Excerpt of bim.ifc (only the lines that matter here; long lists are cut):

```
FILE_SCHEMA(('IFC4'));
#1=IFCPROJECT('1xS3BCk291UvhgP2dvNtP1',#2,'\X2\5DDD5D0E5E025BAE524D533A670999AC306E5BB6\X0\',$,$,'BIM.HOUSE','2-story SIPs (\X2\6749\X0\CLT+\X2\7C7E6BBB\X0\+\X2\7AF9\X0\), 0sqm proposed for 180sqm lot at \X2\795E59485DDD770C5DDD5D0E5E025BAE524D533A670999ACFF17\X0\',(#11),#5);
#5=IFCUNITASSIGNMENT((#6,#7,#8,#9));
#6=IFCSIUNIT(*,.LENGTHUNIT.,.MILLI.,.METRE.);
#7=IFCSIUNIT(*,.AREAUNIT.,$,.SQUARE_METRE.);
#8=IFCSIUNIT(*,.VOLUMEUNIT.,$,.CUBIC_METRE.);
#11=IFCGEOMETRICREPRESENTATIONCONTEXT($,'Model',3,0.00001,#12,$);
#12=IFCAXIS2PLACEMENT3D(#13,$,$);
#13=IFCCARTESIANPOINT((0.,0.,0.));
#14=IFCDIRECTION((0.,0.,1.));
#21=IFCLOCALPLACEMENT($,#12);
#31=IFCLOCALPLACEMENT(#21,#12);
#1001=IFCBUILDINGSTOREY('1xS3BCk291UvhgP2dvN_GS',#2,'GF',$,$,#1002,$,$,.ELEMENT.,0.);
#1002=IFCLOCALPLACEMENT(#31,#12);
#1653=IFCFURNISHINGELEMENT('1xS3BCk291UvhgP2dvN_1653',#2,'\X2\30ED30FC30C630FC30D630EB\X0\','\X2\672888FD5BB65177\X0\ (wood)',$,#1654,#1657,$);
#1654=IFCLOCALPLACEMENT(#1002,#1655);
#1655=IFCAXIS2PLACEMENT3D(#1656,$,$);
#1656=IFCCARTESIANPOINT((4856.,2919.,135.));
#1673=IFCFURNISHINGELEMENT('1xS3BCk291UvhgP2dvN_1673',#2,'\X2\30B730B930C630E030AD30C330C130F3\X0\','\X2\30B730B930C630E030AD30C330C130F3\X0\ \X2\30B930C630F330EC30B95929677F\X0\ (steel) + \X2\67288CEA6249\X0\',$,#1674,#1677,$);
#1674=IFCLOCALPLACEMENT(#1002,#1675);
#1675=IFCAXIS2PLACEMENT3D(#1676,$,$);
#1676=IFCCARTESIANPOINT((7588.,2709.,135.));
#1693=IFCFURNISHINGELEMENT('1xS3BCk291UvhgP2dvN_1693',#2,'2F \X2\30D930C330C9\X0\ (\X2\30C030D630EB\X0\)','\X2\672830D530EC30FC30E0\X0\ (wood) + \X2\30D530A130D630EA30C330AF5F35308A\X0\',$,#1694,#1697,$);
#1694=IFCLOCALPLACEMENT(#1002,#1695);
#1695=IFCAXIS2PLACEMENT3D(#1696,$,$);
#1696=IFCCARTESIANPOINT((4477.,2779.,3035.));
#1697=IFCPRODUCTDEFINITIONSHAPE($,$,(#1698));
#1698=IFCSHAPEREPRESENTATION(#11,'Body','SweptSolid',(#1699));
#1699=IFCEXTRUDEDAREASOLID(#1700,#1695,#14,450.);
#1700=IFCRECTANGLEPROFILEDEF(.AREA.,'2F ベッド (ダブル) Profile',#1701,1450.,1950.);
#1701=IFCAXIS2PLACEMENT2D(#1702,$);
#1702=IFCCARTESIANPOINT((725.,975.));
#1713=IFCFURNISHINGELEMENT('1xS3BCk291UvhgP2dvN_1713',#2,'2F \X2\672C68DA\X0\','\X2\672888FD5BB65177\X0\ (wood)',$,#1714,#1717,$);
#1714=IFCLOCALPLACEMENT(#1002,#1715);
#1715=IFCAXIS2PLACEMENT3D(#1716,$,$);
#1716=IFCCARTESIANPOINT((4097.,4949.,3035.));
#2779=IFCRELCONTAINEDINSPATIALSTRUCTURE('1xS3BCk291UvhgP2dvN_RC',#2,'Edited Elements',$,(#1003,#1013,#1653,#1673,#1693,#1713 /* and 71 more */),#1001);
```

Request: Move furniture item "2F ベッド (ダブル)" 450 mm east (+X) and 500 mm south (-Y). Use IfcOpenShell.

```python
import ifcopenshell
import ifcopenshell.api.geometry
import ifcopenshell.util.placement
import ifcopenshell.util.unit

model = ifcopenshell.open("bim.ifc")
unit_scale = ifcopenshell.util.unit.calculate_unit_scale(model)

item = model.by_guid("1xS3BCk291UvhgP2dvN_1693")
matrix = ifcopenshell.util.placement.get_local_placement(item.ObjectPlacement)
matrix[0, 3] += 0.45 / unit_scale
matrix[1, 3] -= 0.5 / unit_scale
ifcopenshell.api.geometry.edit_object_placement(model, product=item, matrix=matrix, is_si=False)

print(ifcopenshell.util.placement.get_local_placement(item.ObjectPlacement).round(3) + 0.0)

model.write("bim_edited.ifc")
```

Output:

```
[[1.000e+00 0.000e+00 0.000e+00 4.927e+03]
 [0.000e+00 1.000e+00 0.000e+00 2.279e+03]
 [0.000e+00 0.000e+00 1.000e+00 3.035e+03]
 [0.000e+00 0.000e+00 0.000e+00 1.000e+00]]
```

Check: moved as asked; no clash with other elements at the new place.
